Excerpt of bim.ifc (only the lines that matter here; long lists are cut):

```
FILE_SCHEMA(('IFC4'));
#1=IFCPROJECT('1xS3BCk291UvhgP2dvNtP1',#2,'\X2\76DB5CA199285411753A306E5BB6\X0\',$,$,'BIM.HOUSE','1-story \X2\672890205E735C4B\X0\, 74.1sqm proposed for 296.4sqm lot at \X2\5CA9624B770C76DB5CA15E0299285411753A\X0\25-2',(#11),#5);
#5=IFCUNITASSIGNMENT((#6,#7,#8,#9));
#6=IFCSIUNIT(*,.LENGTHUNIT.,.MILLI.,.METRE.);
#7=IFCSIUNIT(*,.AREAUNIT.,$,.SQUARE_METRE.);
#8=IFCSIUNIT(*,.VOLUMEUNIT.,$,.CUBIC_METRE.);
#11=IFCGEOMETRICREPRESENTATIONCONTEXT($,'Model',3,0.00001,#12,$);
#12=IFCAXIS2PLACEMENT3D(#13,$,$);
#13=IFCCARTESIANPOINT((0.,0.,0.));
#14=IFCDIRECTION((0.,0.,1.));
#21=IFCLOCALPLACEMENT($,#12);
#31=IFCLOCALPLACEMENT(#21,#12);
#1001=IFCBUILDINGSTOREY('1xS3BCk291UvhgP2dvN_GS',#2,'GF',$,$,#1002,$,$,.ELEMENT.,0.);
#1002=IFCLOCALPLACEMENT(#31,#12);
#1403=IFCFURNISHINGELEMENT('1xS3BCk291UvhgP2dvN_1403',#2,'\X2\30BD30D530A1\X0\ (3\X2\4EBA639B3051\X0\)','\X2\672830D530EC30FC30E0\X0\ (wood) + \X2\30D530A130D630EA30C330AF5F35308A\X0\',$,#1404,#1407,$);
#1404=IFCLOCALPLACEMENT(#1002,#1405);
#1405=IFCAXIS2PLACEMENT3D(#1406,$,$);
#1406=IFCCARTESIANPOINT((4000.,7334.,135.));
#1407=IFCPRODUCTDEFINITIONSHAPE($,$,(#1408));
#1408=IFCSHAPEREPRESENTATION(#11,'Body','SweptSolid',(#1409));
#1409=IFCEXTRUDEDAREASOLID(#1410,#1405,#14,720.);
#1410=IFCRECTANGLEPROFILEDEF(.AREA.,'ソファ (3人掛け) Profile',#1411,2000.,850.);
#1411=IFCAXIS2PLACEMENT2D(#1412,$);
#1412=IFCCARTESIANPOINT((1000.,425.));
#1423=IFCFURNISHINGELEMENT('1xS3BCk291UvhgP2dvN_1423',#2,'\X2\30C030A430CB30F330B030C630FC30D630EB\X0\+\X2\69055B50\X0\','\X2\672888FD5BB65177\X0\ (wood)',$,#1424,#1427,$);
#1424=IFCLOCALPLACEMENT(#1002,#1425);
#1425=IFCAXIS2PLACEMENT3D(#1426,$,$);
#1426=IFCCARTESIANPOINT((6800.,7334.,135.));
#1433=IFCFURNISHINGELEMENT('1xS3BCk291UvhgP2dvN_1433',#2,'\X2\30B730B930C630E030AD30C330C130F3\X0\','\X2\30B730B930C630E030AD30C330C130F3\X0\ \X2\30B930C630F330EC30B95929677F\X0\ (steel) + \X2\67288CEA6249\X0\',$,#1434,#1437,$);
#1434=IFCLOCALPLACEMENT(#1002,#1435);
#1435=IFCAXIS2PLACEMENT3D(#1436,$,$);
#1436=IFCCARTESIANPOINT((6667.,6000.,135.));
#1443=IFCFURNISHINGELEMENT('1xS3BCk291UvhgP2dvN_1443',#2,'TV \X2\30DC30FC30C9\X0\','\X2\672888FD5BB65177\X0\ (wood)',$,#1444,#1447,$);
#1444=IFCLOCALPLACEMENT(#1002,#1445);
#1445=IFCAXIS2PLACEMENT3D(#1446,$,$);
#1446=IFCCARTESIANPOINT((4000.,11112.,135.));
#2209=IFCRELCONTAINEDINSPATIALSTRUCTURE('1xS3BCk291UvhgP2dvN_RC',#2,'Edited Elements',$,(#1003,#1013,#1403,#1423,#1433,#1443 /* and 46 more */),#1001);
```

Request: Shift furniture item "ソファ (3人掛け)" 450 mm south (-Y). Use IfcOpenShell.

```python
import ifcopenshell
import ifcopenshell.api.geometry
import ifcopenshell.util.placement
import ifcopenshell.util.unit

model = ifcopenshell.open("bim.ifc")
unit_scale = ifcopenshell.util.unit.calculate_unit_scale(model)

item = model.by_guid("1xS3BCk291UvhgP2dvN_1403")
matrix = ifcopenshell.util.placement.get_local_placement(item.ObjectPlacement)
matrix[1, 3] -= 0.45 / unit_scale
ifcopenshell.api.geometry.edit_object_placement(model, product=item, matrix=matrix, is_si=False)

print(ifcopenshell.util.placement.get_local_placement(item.ObjectPlacement).round(3) + 0.0)

model.write("bim-out.ifc")
```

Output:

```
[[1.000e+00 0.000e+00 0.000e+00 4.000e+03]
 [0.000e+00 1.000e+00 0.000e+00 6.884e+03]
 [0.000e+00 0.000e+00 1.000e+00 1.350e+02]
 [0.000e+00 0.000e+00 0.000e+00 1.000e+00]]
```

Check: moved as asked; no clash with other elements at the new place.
